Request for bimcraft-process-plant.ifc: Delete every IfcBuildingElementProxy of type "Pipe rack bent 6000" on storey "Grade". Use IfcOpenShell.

First a look at what the model holds.

```python
import ifcopenshell
import ifcopenshell.util.element

model = ifcopenshell.open("bimcraft-process-plant.ifc")
print(model.schema)
storey = next(s for s in model.by_type("IfcBuildingStorey") if s.Name == "Grade")
proxies = [e for e in ifcopenshell.util.element.get_decomposition(storey) if e.is_a("IfcBuildingElementProxy")]
seen = {}
for e in proxies:
    element_type = ifcopenshell.util.element.get_type(e)
    name = element_type.Name if element_type not in (None, e) else None
    seen[name] = seen.get(name, 0) + 1
for name, count in sorted(seen.items(), key=str):
    print(count, "x", name)
```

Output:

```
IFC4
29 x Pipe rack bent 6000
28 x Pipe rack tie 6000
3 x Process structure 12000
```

```python
import ifcopenshell
import ifcopenshell.api.root
import ifcopenshell.util.element

model = ifcopenshell.open("bimcraft-process-plant.ifc")

storey = next(s for s in model.by_type("IfcBuildingStorey") if s.Name == "Grade")
proxies = [e for e in ifcopenshell.util.element.get_decomposition(storey) if e.is_a("IfcBuildingElementProxy")]
targets = [e for e in proxies if (t := ifcopenshell.util.element.get_type(e)) not in (None, e) and t.Name == "Pipe rack bent 6000"]

for e in targets:
    ifcopenshell.api.root.remove_product(model, product=e)
print(len(targets), "removed")

model.write("bimcraft-process-plant_updated.ifc")
```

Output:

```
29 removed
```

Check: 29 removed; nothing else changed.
